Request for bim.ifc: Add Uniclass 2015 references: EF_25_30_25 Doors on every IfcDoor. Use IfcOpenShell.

First a look at what the model holds.

```python
import ifcopenshell

model = ifcopenshell.open("bim.ifc")
print(model.schema)
print("classifications:", [c.Name for c in model.by_type("IfcClassification")])
for ifc_class in ("IfcDoor", "IfcRoof", "IfcStair", "IfcWall", "IfcWindow"):
    print(ifc_class, len(model.by_type(ifc_class)))
```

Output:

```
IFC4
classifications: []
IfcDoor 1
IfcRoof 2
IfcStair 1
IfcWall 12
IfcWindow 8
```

```python
import ifcopenshell
import ifcopenshell.api.classification

model = ifcopenshell.open("bim.ifc")

system = ifcopenshell.api.classification.add_classification(model, classification="Uniclass 2015")

codes = {
    "IfcDoor": ("EF_25_30_25", "Doors"),
}
for ifc_class, (code, name) in codes.items():
    products = model.by_type(ifc_class)
    ifcopenshell.api.classification.add_reference(
        model, products=products, classification=system, identification=code, name=name
    )
    print(code, len(products))

model.write("bim_v2.ifc")
```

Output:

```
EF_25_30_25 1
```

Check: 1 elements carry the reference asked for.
